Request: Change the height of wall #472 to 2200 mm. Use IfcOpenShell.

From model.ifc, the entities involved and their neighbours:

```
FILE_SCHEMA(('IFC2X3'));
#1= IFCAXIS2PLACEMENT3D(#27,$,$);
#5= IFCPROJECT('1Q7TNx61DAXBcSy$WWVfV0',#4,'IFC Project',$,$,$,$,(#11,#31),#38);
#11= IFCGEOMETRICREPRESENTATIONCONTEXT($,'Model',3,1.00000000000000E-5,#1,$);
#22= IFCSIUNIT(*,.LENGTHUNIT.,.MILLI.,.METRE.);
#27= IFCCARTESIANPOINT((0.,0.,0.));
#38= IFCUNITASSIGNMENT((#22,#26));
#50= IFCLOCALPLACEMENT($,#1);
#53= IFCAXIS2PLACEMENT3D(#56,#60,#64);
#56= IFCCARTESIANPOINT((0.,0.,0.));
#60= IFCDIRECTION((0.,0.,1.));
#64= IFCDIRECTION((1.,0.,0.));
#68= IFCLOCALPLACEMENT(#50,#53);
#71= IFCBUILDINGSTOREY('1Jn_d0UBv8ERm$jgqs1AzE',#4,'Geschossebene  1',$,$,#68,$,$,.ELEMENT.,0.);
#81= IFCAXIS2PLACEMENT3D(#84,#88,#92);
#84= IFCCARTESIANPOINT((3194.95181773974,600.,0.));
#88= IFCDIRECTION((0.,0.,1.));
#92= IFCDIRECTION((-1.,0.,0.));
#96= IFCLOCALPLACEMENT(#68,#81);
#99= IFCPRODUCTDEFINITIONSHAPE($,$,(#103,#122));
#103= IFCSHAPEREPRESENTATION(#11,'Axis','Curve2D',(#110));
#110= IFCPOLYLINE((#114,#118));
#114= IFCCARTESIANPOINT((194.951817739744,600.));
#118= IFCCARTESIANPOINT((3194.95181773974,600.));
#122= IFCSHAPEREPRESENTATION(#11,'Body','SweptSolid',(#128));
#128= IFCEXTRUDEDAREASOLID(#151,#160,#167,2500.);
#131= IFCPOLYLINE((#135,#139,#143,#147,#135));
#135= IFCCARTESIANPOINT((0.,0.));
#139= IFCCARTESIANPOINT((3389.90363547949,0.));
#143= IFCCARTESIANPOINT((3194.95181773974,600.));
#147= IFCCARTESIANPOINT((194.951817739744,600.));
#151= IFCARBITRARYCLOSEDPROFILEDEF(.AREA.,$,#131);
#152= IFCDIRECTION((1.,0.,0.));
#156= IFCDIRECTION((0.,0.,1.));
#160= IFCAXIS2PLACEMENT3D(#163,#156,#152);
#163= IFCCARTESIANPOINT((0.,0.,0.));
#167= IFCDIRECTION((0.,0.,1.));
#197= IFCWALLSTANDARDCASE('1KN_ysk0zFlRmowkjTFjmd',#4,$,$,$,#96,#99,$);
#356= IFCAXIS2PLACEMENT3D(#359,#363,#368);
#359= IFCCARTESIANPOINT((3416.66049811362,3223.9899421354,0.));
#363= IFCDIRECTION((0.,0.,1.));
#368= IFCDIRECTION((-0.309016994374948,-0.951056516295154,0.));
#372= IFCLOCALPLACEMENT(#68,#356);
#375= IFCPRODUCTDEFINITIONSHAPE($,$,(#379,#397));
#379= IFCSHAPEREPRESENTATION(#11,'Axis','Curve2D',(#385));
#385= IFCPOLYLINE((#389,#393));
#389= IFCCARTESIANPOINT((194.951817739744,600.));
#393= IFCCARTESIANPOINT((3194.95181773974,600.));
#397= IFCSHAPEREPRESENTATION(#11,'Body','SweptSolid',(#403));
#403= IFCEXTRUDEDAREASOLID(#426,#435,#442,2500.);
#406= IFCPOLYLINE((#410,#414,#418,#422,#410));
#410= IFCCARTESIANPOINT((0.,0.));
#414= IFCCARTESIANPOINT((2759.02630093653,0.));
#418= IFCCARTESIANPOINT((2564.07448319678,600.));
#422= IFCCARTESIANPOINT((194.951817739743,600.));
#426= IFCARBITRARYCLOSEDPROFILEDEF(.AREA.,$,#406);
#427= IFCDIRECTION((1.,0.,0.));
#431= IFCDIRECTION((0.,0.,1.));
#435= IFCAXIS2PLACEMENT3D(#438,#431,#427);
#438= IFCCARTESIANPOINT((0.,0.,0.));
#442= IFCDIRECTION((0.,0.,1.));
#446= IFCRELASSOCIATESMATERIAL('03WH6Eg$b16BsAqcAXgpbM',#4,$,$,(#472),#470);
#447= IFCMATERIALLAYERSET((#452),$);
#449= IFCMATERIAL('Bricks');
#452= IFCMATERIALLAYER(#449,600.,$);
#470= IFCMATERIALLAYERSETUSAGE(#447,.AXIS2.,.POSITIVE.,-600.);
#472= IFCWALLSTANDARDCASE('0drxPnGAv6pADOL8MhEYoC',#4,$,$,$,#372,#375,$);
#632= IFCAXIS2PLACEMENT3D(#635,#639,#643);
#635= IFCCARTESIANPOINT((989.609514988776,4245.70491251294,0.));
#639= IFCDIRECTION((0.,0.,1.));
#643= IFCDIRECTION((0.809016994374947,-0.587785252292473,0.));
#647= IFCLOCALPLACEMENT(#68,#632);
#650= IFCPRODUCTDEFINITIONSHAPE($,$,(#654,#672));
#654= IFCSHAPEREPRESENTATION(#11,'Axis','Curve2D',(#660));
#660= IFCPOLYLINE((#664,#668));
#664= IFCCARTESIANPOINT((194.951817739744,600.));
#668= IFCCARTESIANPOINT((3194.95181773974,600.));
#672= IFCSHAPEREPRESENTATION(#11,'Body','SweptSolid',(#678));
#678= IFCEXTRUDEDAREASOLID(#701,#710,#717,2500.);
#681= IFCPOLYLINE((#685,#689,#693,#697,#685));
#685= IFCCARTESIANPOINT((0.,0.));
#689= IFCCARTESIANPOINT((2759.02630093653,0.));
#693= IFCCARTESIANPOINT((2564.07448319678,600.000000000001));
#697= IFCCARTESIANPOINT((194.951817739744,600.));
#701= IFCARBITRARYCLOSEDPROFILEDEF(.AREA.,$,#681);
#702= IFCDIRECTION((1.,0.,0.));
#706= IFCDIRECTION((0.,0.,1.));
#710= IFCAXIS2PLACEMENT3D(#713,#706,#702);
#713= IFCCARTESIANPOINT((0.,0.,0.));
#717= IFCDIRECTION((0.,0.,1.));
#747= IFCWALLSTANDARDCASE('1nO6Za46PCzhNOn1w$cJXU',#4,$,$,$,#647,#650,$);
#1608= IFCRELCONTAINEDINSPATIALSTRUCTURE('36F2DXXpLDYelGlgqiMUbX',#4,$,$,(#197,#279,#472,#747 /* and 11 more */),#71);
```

```python
import ifcopenshell
import ifcopenshell.geom
import ifcopenshell.util.shape
import ifcopenshell.util.unit

model = ifcopenshell.open("model.ifc")
unit_scale = ifcopenshell.util.unit.calculate_unit_scale(model)
settings = ifcopenshell.geom.settings()


def volume(element):
    """Net volume in cubic metres, openings subtracted."""
    shape = ifcopenshell.geom.create_shape(settings, element)
    return ifcopenshell.util.shape.get_volume(shape.geometry)


wall = model.by_guid("0drxPnGAv6pADOL8MhEYoC")
before = volume(wall)

body = next(r for r in wall.Representation.Representations if r.RepresentationIdentifier == "Body")
solid = body.Items[0]
old_height = solid.Depth
solid.Depth = 2.2 / unit_scale
after = volume(wall)

print(f"height {old_height:g} -> {solid.Depth:g}, volume {before:.3f} -> {after:.3f} m3")

model.write("model_edited.ifc")
```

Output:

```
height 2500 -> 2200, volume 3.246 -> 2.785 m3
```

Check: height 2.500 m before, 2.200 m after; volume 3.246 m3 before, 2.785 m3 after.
